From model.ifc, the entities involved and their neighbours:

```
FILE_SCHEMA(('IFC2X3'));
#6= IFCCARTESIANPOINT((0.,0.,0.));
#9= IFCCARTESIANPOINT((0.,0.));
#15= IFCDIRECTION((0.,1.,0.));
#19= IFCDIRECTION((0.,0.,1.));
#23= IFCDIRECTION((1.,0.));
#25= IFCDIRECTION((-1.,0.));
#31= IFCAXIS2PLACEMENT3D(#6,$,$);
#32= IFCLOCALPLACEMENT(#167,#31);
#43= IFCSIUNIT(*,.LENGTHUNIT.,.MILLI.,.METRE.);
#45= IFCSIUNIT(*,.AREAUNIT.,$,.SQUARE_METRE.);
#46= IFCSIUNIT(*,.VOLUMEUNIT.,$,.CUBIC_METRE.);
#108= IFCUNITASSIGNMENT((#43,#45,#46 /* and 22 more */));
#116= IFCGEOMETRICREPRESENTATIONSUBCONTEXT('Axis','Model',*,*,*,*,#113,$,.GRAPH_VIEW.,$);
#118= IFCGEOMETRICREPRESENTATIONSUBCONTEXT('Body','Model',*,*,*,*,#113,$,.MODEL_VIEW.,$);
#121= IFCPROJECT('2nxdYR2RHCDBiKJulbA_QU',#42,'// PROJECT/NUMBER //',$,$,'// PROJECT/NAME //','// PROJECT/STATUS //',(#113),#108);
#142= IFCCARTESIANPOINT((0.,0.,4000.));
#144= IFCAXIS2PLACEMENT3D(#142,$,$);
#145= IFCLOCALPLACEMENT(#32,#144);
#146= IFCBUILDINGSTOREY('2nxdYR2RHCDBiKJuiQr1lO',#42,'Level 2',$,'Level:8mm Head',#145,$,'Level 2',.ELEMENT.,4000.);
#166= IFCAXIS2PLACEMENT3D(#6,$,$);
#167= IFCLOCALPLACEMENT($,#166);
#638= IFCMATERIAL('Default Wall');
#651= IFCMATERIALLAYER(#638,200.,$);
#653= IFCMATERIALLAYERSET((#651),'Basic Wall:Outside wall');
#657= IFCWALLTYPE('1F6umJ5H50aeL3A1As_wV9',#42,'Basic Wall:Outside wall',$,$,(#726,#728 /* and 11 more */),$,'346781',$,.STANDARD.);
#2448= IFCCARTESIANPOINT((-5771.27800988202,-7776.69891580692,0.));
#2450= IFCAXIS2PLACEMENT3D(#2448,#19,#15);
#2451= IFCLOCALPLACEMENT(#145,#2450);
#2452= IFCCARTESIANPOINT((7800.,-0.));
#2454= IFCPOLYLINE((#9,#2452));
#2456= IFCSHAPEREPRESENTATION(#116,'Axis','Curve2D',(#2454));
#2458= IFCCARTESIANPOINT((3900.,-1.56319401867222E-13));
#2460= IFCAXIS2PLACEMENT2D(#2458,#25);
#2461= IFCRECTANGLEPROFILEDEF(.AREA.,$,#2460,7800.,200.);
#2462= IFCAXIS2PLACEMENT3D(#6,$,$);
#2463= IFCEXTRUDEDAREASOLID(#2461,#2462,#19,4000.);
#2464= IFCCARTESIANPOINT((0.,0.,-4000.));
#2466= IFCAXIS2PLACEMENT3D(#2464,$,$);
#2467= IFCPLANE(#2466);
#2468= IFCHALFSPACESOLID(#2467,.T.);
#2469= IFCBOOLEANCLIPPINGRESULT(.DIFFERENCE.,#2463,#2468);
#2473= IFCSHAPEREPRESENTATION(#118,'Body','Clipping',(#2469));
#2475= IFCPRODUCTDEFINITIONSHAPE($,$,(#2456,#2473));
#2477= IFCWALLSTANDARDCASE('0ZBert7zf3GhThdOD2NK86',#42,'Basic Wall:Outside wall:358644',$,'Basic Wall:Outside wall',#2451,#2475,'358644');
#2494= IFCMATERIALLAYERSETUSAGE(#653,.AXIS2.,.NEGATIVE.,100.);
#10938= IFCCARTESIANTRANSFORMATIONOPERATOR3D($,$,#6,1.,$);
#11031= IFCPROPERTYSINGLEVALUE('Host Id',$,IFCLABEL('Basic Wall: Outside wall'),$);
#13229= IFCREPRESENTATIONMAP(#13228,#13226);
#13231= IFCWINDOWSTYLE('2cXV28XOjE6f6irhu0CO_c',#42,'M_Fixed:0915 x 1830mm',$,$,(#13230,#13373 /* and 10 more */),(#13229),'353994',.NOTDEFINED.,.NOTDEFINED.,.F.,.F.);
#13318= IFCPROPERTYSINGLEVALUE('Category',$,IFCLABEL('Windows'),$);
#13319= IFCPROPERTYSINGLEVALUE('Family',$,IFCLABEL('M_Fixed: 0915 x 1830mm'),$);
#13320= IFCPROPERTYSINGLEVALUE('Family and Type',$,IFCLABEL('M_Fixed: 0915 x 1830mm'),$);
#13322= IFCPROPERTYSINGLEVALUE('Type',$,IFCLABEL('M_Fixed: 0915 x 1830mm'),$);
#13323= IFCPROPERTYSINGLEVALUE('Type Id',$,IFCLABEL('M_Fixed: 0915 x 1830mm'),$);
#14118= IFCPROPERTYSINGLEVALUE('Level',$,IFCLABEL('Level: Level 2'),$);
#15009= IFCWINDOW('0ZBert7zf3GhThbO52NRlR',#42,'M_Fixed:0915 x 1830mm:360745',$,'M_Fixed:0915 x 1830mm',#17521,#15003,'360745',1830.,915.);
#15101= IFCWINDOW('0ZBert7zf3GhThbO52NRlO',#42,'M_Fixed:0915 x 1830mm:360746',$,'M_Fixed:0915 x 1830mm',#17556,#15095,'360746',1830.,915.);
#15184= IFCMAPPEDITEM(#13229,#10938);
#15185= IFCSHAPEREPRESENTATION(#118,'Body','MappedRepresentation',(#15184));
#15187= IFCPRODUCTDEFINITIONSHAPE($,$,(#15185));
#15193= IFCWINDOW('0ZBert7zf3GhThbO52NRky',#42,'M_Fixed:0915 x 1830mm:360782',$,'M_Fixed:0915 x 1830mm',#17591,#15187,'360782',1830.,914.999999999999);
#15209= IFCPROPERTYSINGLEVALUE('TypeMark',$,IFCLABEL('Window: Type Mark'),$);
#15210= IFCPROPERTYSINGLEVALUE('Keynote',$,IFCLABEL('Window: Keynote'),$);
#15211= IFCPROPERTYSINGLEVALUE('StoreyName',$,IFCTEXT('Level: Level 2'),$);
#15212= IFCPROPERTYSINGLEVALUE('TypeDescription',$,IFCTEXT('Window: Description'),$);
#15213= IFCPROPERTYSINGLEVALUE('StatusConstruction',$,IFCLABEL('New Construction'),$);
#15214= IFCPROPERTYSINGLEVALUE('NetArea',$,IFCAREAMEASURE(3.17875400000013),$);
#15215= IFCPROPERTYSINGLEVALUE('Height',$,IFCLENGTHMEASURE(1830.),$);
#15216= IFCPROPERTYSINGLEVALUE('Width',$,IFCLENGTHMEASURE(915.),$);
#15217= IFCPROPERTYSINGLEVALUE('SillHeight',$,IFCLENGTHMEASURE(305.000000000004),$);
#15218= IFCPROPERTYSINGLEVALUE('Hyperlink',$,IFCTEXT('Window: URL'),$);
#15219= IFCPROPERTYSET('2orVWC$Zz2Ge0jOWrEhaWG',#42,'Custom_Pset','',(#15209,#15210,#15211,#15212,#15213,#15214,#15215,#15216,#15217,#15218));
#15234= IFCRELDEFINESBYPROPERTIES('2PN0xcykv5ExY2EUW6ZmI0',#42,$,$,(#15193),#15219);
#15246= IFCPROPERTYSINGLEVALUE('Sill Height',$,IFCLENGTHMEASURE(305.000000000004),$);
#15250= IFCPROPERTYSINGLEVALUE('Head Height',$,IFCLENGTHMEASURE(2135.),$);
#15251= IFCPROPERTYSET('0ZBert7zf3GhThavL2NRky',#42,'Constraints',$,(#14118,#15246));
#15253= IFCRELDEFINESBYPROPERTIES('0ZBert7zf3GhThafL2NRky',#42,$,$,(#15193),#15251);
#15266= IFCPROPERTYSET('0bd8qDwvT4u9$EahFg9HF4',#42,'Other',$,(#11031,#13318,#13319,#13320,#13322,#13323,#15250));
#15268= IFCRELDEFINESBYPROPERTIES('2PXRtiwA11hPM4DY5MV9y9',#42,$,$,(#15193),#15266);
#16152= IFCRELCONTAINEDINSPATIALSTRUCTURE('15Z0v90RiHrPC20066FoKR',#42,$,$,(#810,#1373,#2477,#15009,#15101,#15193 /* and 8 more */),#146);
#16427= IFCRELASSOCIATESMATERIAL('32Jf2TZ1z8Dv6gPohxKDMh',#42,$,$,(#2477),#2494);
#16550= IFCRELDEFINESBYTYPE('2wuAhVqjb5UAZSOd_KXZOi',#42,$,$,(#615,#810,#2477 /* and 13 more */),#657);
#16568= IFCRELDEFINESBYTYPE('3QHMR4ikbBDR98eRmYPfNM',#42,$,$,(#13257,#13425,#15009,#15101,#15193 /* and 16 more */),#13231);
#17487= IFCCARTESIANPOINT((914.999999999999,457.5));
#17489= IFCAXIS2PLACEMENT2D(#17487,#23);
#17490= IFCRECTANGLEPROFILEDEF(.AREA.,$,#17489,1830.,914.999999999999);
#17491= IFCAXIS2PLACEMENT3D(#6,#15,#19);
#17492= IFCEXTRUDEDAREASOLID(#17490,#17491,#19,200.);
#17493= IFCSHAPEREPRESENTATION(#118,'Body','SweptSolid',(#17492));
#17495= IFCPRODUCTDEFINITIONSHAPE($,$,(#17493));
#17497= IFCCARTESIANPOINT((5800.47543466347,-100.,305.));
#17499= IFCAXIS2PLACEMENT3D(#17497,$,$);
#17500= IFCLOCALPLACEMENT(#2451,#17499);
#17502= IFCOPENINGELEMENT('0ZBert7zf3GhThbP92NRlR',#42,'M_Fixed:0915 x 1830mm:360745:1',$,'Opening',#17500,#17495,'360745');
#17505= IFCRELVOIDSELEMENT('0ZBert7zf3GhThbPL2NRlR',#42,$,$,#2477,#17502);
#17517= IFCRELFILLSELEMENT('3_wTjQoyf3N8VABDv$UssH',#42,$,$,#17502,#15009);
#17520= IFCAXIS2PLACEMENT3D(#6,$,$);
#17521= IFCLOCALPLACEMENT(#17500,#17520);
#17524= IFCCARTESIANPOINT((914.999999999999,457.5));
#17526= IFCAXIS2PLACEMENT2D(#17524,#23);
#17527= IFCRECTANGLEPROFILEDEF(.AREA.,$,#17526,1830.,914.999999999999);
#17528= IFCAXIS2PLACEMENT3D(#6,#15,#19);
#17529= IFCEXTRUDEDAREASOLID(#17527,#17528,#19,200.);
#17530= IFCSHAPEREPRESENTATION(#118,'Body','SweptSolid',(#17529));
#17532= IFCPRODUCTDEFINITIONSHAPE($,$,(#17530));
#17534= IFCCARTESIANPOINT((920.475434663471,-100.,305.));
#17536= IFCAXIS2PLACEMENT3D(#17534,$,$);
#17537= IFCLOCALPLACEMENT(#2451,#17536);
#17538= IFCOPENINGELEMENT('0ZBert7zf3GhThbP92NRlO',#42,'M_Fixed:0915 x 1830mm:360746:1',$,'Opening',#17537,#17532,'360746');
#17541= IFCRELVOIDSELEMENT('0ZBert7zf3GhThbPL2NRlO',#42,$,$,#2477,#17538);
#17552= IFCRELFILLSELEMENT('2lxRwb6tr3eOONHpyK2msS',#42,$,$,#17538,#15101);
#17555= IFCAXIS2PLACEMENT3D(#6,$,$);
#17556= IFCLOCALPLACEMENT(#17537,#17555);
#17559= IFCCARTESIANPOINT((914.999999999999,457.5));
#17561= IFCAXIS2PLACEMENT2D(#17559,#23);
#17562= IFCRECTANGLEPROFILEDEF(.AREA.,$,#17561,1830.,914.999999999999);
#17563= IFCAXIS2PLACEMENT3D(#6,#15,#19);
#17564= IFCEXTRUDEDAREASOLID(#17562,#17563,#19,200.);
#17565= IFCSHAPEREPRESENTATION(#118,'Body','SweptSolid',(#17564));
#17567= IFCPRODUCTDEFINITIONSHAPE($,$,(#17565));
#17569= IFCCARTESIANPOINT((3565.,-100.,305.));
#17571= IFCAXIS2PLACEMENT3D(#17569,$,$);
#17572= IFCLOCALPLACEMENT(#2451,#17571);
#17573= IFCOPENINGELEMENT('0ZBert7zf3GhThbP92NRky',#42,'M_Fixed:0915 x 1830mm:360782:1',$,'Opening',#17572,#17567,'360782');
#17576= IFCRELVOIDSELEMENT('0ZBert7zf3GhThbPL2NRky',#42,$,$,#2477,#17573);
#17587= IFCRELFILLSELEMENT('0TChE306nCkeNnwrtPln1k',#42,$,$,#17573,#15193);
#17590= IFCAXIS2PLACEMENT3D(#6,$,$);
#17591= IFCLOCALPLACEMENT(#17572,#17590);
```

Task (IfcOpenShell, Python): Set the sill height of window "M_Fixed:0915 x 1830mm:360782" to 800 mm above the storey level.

```python
import numpy as np
import ifcopenshell
import ifcopenshell.api.geometry
import ifcopenshell.api.pset
import ifcopenshell.geom
import ifcopenshell.util.element
import ifcopenshell.util.placement
import ifcopenshell.util.shape
import ifcopenshell.util.unit

model = ifcopenshell.open("model.ifc")
unit_scale = ifcopenshell.util.unit.calculate_unit_scale(model)

window = model.by_guid("0ZBert7zf3GhThbO52NRky")
opening = window.FillsVoids[0].RelatingOpeningElement
storey = ifcopenshell.util.element.get_container(window, ifc_class="IfcBuildingStorey")
level = ifcopenshell.util.placement.get_local_placement(storey.ObjectPlacement)[2, 3]

# The opening's origin need not be at the sill, so measure its lowest point.
shape = ifcopenshell.geom.create_shape(ifcopenshell.geom.settings(), opening)
bottom = ifcopenshell.util.shape.get_shape_bottom_elevation(shape, shape.geometry) / unit_scale
dz = level + 800.0 - bottom

shift = np.array([0.0, 0.0, dz])
# The window is placed relative to its opening, so it follows when the opening moves.
matrix = ifcopenshell.util.placement.get_local_placement(opening.ObjectPlacement)
matrix[:3, 3] += shift
ifcopenshell.api.geometry.edit_object_placement(
    model, product=opening, matrix=matrix, is_si=False, should_transform_children=True
)

# Keep the stored heights in step.
pset = model.by_id(ifcopenshell.util.element.get_pset(window, "Custom_Pset", should_inherit=False)["id"])
ifcopenshell.api.pset.edit_pset(model, pset=pset, properties={
    "SillHeight": model.create_entity("IfcLengthMeasure", ifcopenshell.util.element.get_pset(window, "Constraints", "Sill Height") + dz),
})
pset = model.by_id(ifcopenshell.util.element.get_pset(window, "Constraints", should_inherit=False)["id"])
ifcopenshell.api.pset.edit_pset(model, pset=pset, properties={
    "Sill Height": model.create_entity("IfcLengthMeasure", ifcopenshell.util.element.get_pset(window, "Constraints", "Sill Height") + dz),
})
pset = model.by_id(ifcopenshell.util.element.get_pset(window, "Other", should_inherit=False)["id"])
ifcopenshell.api.pset.edit_pset(model, pset=pset, properties={
    "Head Height": model.create_entity("IfcLengthMeasure", ifcopenshell.util.element.get_pset(window, "Other", "Head Height") + dz),
})

print(f"moved by {dz * unit_scale:+.3f} m")

model.write("model_updated.ifc")
```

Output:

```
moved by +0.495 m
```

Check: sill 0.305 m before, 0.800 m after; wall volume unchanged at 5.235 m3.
